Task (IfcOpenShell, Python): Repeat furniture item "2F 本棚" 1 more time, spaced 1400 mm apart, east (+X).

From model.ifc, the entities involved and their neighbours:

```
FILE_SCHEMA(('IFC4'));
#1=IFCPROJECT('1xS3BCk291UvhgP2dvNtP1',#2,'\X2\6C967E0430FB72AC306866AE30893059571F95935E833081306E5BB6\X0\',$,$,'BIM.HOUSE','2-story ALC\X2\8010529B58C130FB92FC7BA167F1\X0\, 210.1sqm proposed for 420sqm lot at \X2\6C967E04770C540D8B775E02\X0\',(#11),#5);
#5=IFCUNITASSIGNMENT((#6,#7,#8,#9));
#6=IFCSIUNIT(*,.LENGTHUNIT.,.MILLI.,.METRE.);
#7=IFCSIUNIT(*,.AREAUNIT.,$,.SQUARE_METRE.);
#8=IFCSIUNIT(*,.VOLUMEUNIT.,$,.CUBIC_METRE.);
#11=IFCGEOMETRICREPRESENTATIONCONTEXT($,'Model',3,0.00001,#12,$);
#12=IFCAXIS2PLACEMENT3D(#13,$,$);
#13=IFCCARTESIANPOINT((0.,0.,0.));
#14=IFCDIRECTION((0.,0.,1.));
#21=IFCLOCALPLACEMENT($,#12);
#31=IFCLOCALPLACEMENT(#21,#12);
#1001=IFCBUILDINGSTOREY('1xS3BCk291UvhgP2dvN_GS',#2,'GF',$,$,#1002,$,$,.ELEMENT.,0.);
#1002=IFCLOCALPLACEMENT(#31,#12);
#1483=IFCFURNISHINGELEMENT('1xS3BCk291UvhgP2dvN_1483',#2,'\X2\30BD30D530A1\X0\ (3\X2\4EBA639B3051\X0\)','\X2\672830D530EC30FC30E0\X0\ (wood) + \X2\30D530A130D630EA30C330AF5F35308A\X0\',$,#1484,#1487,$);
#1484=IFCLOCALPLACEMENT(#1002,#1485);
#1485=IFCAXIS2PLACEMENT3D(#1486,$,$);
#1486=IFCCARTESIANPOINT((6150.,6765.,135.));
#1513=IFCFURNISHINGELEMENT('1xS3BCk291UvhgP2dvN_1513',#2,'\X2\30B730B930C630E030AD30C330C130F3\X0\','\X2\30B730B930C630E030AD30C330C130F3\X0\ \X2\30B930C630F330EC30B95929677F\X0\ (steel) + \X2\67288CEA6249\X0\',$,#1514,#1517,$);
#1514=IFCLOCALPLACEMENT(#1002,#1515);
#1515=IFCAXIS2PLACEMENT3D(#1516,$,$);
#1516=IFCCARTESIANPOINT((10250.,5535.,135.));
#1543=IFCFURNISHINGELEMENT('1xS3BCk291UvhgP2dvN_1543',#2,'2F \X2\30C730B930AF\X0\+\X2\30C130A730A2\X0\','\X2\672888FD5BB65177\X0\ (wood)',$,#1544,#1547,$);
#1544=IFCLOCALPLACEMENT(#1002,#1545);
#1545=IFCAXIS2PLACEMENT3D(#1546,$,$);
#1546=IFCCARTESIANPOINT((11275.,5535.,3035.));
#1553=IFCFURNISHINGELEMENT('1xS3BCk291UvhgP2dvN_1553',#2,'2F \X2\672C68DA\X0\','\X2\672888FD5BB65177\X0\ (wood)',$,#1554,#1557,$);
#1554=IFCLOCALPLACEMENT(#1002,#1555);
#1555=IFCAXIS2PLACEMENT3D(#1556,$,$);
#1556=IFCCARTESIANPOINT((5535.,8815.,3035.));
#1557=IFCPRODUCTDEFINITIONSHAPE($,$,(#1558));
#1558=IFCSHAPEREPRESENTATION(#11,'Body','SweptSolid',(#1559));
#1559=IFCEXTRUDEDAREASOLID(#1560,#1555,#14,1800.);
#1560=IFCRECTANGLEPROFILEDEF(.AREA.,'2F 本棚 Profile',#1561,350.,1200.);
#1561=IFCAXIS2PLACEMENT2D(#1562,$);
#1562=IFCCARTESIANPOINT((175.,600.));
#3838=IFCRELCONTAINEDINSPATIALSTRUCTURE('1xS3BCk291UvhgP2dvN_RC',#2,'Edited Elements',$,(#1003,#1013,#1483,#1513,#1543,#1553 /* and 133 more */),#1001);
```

```python
import numpy as np
import ifcopenshell
import ifcopenshell.api.geometry
import ifcopenshell.api.root
import ifcopenshell.util.element
import ifcopenshell.util.placement
import ifcopenshell.util.unit

model = ifcopenshell.open("model.ifc")
unit_scale = ifcopenshell.util.unit.calculate_unit_scale(model)


def reuse_history(source, copy):
    """copy_class also copies each property set's owner history, people and application; keep the originals."""
    for rel in copy.IsDefinedBy:
        if rel.is_a("IfcRelDefinesByProperties") and (history := rel.RelatingPropertyDefinition.OwnerHistory):
            rel.RelatingPropertyDefinition.OwnerHistory = source.OwnerHistory
            ifcopenshell.util.element.remove_deep2(model, history)


source = model.by_id(1553)
base = ifcopenshell.util.placement.get_local_placement(source.ObjectPlacement)
step = np.array([1.0, 0.0, 0.0]) * 1.4 / unit_scale

for i in range(1, 2):
    copy = ifcopenshell.api.root.copy_class(model, product=source)
    copy.Representation = ifcopenshell.util.element.copy_deep(
        model, source.Representation, exclude=["IfcGeometricRepresentationContext", "IfcRepresentationMap"]
    )
    reuse_history(source, copy)
    matrix = base.copy()
    matrix[:3, 3] += i * step
    print("added at", matrix[:3, 3].round(3) + 0.0)
    ifcopenshell.api.geometry.edit_object_placement(model, product=copy, matrix=matrix, is_si=False)

model.write("model_updated.ifc")
```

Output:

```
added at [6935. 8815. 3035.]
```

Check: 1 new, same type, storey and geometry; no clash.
